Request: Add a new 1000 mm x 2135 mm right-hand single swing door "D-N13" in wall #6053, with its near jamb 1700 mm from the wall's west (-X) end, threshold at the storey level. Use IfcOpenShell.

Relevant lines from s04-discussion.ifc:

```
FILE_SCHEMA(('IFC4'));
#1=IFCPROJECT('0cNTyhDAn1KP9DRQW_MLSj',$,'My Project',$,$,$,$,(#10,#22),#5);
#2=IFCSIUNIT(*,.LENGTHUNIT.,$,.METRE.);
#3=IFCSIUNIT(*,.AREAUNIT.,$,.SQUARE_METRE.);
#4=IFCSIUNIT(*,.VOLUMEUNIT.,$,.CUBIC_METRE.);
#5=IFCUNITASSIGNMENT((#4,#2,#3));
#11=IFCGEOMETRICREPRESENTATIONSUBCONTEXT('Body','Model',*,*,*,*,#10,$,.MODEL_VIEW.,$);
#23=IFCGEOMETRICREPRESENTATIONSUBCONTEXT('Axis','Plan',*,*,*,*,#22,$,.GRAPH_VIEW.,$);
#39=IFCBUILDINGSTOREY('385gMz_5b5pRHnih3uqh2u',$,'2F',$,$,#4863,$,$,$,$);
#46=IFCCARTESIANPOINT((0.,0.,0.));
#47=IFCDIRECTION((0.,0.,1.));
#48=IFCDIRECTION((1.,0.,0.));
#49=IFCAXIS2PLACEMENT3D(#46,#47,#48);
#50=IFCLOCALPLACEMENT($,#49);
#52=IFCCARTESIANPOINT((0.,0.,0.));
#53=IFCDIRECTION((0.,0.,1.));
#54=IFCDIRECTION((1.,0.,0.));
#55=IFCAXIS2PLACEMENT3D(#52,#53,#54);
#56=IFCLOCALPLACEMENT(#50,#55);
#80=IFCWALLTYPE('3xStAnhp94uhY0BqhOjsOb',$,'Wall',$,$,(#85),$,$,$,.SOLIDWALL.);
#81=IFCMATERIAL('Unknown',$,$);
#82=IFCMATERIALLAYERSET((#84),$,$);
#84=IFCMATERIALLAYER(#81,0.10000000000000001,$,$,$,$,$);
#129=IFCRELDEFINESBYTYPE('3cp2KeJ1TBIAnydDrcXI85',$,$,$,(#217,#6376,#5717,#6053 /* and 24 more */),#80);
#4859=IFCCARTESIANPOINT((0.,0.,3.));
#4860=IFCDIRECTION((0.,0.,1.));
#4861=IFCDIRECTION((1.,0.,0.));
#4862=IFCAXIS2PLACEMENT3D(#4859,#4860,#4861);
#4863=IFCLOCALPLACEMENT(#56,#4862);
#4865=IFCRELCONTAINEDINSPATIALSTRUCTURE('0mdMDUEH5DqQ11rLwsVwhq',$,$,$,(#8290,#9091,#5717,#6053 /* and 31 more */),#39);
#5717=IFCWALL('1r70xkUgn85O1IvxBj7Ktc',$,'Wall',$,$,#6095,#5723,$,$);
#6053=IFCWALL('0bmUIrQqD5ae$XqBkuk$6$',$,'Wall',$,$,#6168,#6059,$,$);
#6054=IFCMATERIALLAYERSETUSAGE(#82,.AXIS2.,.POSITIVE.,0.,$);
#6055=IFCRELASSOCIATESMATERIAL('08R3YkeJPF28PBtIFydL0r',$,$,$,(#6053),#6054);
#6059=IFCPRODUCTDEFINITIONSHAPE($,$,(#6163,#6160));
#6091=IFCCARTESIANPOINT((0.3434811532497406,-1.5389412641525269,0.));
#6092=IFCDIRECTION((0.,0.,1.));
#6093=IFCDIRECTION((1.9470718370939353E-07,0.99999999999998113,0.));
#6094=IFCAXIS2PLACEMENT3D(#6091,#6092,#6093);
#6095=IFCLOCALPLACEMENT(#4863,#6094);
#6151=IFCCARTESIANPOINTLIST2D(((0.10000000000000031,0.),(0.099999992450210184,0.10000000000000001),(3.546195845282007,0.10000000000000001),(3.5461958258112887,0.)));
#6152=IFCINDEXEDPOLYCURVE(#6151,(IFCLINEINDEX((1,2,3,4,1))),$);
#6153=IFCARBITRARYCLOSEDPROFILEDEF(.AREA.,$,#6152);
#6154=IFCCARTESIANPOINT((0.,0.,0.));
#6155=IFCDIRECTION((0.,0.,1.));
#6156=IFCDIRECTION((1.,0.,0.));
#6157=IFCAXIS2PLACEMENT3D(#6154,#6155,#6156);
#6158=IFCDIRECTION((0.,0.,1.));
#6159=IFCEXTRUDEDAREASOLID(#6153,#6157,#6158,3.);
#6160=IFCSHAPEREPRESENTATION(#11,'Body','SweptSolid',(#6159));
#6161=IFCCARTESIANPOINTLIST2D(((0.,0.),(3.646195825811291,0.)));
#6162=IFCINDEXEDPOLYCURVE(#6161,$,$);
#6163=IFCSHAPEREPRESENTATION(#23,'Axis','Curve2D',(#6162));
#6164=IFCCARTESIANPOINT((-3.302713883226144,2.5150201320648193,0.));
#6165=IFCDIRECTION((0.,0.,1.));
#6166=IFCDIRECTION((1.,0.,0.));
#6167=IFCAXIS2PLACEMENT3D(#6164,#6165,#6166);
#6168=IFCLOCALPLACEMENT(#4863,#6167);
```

```python
import numpy as np
import ifcopenshell
import ifcopenshell.api.feature
import ifcopenshell.api.geometry
import ifcopenshell.api.root
import ifcopenshell.api.spatial
import ifcopenshell.geom
import ifcopenshell.util.element
import ifcopenshell.util.placement
import ifcopenshell.util.representation
import ifcopenshell.util.shape
import ifcopenshell.util.unit

model = ifcopenshell.open("s04-discussion.ifc")
unit_scale = ifcopenshell.util.unit.calculate_unit_scale(model)
settings = ifcopenshell.geom.settings()


def volume(element):
    """Net volume in cubic metres, openings subtracted."""
    shape = ifcopenshell.geom.create_shape(settings, element)
    return ifcopenshell.util.shape.get_volume(shape.geometry)


wall = model.by_guid("0bmUIrQqD5ae$XqBkuk$6$")
storey = ifcopenshell.util.element.get_container(wall, ifc_class="IfcBuildingStorey")
context = ifcopenshell.util.representation.get_context(model, "Model", "Body", "MODEL_VIEW")
before = volume(wall)

width, height, from_end, sill = 1, 2.135, 1.7, 0.0  # metres

# The wall runs along its own X axis, and the end named is its -X end.
wall_shape = ifcopenshell.geom.create_shape(settings, wall)
x, y, z = ifcopenshell.util.shape.get_vertices(wall_shape.geometry).T
start = x.min() + from_end
face, thickness = float(y.min()), float(y.max() - y.min())
wall_matrix = ifcopenshell.util.placement.get_local_placement(wall.ObjectPlacement)
level = ifcopenshell.util.placement.get_local_placement(storey.ObjectPlacement)[2, 3]


def in_wall(x, y):
    """Placement at x, y metres in the wall's axes, at sill height."""
    matrix = wall_matrix.copy()
    matrix[:, 3] = wall_matrix @ np.array([x / unit_scale, y / unit_scale, 0.0, 1.0])
    matrix[2, 3] = level + sill / unit_scale
    return matrix


# Opening: a box that overshoots both wall faces by 50 mm.
opening = ifcopenshell.api.root.create_entity(model, ifc_class="IfcOpeningElement", predefined_type="OPENING")
box = ifcopenshell.api.geometry.add_wall_representation(
    model, context=context, length=width, height=height, thickness=thickness + 0.1
)
ifcopenshell.api.geometry.assign_representation(model, product=opening, representation=box)
ifcopenshell.api.geometry.edit_object_placement(model, product=opening, matrix=in_wall(start, face - 0.05), is_si=False)
ifcopenshell.api.feature.add_feature(model, feature=opening, element=wall)

door = ifcopenshell.api.root.create_entity(model, ifc_class="IfcDoor", name="D-N13", predefined_type="DOOR")
door.OverallWidth, door.OverallHeight = width / unit_scale, height / unit_scale
door.OperationType = "SINGLE_SWING_RIGHT"
body = ifcopenshell.api.geometry.add_door_representation(
    model,
    context=context,
    overall_width=door.OverallWidth,
    overall_height=door.OverallHeight,
    operation_type="SINGLE_SWING_RIGHT",
    lining_properties={"LiningDepth": thickness / unit_scale, "ThresholdDepth": thickness / unit_scale},
)
ifcopenshell.api.geometry.assign_representation(model, product=door, representation=body)
ifcopenshell.api.spatial.assign_container(model, products=[door], relating_structure=storey)
ifcopenshell.api.feature.add_filling(model, opening=opening, element=door)

# The lining spans the wall, so the door starts at the wall face.
ifcopenshell.api.geometry.edit_object_placement(model, product=door, matrix=in_wall(start, face), is_si=False)

after = volume(wall)

print(f"wall volume {before:.3f} -> {after:.3f} m3")

model.write("s04-discussion_rev.ifc")
```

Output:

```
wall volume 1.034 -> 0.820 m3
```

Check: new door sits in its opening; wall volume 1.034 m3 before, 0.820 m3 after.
